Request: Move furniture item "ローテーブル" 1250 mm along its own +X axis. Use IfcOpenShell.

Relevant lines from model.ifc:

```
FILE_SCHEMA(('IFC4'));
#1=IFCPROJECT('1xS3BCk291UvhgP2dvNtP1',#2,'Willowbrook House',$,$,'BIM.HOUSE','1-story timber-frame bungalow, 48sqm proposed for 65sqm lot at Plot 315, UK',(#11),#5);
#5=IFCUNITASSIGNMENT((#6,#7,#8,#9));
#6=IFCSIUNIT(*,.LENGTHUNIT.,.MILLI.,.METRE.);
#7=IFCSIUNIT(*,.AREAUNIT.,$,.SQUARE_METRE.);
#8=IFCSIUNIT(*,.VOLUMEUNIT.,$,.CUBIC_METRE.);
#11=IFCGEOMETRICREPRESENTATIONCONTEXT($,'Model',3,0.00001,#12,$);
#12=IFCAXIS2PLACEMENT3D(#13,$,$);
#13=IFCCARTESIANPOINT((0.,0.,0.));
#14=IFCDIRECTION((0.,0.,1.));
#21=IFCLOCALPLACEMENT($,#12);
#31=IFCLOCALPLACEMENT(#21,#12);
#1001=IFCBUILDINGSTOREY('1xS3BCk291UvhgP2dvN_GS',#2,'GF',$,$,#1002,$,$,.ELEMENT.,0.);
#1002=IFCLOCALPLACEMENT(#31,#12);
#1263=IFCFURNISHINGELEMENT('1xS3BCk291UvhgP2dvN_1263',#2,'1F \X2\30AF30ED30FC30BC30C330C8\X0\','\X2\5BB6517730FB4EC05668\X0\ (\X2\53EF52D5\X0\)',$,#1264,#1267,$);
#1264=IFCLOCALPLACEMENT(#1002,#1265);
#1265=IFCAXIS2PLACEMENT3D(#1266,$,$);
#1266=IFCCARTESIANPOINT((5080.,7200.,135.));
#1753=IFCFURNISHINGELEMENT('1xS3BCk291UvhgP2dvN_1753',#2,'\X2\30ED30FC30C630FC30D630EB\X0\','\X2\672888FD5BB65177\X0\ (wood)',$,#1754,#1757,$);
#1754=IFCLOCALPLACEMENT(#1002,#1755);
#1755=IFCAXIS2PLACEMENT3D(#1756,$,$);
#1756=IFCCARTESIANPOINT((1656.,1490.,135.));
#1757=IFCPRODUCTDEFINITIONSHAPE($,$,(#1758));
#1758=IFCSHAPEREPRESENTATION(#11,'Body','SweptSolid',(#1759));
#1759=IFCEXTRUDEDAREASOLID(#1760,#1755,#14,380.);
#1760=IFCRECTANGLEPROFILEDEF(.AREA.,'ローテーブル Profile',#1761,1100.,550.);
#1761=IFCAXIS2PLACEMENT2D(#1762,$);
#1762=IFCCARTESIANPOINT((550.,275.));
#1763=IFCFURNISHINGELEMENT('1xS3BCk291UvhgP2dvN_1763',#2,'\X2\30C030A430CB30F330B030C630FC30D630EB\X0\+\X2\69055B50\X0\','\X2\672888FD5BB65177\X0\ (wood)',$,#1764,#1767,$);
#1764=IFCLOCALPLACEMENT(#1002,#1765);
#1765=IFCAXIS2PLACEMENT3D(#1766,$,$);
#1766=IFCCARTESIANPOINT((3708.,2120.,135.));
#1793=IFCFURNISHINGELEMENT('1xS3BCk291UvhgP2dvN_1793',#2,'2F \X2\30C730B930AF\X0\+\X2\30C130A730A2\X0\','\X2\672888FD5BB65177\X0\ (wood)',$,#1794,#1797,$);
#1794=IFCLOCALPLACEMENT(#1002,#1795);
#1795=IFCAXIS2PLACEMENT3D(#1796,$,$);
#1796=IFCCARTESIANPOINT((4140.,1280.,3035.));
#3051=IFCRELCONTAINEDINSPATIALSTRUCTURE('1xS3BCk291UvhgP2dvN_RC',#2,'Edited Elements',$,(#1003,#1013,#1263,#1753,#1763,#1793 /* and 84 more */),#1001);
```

```python
import ifcopenshell
import ifcopenshell.api.geometry
import ifcopenshell.util.placement

model = ifcopenshell.open("model.ifc")

item = model.by_guid("1xS3BCk291UvhgP2dvN_1753")
matrix = ifcopenshell.util.placement.get_local_placement(item.ObjectPlacement)
matrix[:3, 3] += matrix[:3, 0] * 1250.0
ifcopenshell.api.geometry.edit_object_placement(model, product=item, matrix=matrix, is_si=False)

print(ifcopenshell.util.placement.get_local_placement(item.ObjectPlacement).round(3) + 0.0)

model.write("model_v2.ifc")
```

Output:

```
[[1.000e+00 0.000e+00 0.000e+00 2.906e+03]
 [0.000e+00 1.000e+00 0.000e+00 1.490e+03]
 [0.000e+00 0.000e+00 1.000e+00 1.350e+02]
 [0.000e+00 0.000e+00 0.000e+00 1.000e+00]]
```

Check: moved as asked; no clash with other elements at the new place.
